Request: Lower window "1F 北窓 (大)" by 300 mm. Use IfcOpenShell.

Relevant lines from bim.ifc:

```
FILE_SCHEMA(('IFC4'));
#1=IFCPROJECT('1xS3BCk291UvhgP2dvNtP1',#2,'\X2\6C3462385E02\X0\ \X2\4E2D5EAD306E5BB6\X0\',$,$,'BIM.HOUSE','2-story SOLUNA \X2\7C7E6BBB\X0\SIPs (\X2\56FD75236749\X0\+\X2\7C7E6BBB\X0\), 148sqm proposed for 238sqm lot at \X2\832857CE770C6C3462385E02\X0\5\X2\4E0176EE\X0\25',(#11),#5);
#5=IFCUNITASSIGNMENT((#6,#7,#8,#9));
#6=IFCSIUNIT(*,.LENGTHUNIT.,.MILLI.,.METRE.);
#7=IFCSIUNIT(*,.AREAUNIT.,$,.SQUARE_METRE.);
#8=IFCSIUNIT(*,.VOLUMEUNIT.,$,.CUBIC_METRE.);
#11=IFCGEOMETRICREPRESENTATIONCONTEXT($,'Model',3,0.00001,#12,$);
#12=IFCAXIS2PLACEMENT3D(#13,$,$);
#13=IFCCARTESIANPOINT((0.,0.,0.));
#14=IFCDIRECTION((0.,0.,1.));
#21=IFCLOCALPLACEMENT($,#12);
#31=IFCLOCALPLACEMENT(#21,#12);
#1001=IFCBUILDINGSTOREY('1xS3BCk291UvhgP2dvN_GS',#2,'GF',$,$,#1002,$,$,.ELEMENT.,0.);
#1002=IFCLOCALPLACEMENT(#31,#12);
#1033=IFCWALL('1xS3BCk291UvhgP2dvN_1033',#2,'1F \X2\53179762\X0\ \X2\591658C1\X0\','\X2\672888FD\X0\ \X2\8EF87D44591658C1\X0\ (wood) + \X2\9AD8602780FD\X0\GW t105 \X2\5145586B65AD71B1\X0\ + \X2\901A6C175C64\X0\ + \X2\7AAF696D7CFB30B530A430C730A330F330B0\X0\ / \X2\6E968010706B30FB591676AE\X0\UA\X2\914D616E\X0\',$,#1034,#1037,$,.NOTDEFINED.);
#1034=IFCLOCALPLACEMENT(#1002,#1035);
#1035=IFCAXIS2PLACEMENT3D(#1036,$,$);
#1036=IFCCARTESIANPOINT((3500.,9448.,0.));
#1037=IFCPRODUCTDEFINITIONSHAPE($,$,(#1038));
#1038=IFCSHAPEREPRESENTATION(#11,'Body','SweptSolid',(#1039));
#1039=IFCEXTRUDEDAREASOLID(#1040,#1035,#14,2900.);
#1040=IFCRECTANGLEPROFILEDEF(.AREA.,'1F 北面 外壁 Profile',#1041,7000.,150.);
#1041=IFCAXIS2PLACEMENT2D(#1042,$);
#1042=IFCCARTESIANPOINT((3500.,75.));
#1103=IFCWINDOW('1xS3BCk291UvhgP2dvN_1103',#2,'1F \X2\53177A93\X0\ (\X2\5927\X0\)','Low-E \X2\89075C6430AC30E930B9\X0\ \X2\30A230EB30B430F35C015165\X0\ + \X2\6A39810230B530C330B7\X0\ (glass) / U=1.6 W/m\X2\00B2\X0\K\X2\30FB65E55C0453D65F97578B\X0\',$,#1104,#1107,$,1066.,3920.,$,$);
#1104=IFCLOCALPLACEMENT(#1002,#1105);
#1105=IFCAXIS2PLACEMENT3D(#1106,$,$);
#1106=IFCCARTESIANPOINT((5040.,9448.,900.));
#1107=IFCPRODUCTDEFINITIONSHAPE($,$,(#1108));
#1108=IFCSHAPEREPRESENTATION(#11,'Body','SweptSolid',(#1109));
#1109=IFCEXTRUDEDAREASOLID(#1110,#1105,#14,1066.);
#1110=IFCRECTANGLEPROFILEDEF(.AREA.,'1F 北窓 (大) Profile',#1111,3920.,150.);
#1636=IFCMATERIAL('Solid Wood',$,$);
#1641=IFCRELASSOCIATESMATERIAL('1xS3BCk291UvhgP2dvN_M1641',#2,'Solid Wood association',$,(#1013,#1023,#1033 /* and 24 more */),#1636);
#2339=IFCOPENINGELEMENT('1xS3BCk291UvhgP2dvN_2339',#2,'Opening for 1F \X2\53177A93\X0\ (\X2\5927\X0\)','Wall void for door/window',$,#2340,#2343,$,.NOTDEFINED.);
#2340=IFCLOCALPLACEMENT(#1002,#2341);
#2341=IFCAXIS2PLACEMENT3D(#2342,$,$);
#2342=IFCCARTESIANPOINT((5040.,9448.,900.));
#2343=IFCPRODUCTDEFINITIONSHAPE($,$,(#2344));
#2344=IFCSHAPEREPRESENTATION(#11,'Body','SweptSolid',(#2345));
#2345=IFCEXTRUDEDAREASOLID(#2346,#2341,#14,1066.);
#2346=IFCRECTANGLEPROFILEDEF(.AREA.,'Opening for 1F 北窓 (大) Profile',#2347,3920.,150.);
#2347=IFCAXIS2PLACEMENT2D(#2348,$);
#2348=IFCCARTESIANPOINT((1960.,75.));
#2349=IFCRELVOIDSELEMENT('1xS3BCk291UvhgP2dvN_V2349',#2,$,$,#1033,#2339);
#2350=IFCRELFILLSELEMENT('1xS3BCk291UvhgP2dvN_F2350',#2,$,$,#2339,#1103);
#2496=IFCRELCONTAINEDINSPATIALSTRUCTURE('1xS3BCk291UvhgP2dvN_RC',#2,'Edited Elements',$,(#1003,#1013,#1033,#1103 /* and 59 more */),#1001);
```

```python
import numpy as np
import ifcopenshell
import ifcopenshell.api.geometry
import ifcopenshell.util.placement
import ifcopenshell.util.unit

model = ifcopenshell.open("bim.ifc")
unit_scale = ifcopenshell.util.unit.calculate_unit_scale(model)

window = model.by_id(1103)
opening = window.FillsVoids[0].RelatingOpeningElement
dz = -0.3 / unit_scale

shift = np.array([0.0, 0.0, dz])
# The window is not placed relative to its opening, so move both.
for product in (opening, window):
    matrix = ifcopenshell.util.placement.get_local_placement(product.ObjectPlacement)
    matrix[:3, 3] += shift
    ifcopenshell.api.geometry.edit_object_placement(model, product=product, matrix=matrix, is_si=False)

print(f"moved by {dz * unit_scale:+.3f} m")

model.write("bim_updated.ifc")
```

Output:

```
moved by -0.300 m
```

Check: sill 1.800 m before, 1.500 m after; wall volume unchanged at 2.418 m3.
